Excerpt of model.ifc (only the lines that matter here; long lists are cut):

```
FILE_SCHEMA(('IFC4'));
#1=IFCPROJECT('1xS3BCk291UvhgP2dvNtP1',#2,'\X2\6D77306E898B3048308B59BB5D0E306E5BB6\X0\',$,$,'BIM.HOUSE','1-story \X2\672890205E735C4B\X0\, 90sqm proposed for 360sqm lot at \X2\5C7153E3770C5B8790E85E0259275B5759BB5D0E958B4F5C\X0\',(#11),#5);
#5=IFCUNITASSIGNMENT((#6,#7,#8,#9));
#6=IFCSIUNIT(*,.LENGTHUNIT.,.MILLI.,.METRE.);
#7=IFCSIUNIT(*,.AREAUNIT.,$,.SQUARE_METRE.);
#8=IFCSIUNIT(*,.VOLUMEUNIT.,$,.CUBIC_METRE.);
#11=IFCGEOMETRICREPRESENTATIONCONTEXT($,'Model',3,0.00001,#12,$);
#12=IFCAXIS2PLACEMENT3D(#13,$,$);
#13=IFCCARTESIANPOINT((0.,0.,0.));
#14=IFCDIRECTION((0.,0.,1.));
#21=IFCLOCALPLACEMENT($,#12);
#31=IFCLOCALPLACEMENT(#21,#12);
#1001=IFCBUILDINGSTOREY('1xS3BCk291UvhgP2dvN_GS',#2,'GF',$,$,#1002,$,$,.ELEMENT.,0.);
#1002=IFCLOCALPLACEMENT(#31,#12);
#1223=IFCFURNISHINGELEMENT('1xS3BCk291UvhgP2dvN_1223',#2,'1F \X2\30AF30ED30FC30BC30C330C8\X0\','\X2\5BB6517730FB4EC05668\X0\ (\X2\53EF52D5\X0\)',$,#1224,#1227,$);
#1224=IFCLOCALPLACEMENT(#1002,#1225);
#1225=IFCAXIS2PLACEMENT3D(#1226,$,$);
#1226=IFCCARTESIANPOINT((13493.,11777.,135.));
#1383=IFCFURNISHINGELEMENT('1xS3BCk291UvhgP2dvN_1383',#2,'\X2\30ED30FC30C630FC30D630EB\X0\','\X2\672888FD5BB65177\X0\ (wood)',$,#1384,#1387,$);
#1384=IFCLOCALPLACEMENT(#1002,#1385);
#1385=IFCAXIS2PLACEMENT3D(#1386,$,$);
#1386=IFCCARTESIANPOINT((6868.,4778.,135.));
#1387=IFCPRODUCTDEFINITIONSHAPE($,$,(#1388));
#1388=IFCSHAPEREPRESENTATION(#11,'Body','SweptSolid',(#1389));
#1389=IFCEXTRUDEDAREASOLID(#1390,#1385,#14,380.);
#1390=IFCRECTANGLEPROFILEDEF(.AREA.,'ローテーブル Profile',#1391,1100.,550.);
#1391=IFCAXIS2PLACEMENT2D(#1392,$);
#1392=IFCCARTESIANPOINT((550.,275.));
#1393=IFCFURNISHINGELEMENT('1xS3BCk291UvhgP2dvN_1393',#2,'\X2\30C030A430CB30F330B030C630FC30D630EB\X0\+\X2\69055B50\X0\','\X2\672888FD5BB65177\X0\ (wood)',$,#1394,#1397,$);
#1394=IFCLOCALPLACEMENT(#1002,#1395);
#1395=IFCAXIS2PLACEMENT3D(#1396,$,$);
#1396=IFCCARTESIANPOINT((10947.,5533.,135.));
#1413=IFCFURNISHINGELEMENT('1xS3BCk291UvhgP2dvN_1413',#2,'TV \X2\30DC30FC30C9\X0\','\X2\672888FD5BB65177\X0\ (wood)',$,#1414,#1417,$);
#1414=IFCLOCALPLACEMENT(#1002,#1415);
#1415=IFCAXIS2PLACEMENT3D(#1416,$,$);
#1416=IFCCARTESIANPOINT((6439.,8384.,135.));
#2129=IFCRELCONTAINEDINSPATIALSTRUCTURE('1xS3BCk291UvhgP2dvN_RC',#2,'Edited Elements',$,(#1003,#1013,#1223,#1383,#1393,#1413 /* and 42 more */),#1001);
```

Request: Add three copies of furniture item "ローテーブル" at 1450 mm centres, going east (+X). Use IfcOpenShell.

```python
import numpy as np
import ifcopenshell
import ifcopenshell.api.geometry
import ifcopenshell.api.root
import ifcopenshell.util.element
import ifcopenshell.util.placement
import ifcopenshell.util.unit

model = ifcopenshell.open("model.ifc")
unit_scale = ifcopenshell.util.unit.calculate_unit_scale(model)


def reuse_history(source, copy):
    """copy_class also copies each property set's owner history, people and application; keep the originals."""
    for rel in copy.IsDefinedBy:
        if rel.is_a("IfcRelDefinesByProperties") and (history := rel.RelatingPropertyDefinition.OwnerHistory):
            rel.RelatingPropertyDefinition.OwnerHistory = source.OwnerHistory
            ifcopenshell.util.element.remove_deep2(model, history)


source = model.by_id(1383)
base = ifcopenshell.util.placement.get_local_placement(source.ObjectPlacement)
step = np.array([1.0, 0.0, 0.0]) * 1.45 / unit_scale

for i in range(1, 4):
    copy = ifcopenshell.api.root.copy_class(model, product=source)
    copy.Representation = ifcopenshell.util.element.copy_deep(
        model, source.Representation, exclude=["IfcGeometricRepresentationContext", "IfcRepresentationMap"]
    )
    reuse_history(source, copy)
    matrix = base.copy()
    matrix[:3, 3] += i * step
    print("added at", matrix[:3, 3].round(3) + 0.0)
    ifcopenshell.api.geometry.edit_object_placement(model, product=copy, matrix=matrix, is_si=False)

model.write("model_edited.ifc")
```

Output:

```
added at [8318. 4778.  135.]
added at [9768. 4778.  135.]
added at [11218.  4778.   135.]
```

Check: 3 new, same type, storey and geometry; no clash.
